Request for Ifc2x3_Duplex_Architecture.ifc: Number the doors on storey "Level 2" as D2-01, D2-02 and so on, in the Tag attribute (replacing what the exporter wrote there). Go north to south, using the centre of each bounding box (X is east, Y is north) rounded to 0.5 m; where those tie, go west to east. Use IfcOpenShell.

First a look at what the model holds.

```python
import ifcopenshell
import ifcopenshell.util.element
import ifcopenshell.util.placement

model = ifcopenshell.open("Ifc2x3_Duplex_Architecture.ifc")
print(model.schema)
storey = next(s for s in model.by_type("IfcBuildingStorey") if s.Name == "Level 2")
doors = [e for e in ifcopenshell.util.element.get_decomposition(storey) if e.is_a("IfcDoor")]
for e in sorted(doors, key=lambda e: e.id()):
    origin = ifcopenshell.util.placement.get_local_placement(e.ObjectPlacement)[:3, 3]
    print(e.id(), e.Tag, e.Name, origin.round(2) + 0.0, sep=" | ")
```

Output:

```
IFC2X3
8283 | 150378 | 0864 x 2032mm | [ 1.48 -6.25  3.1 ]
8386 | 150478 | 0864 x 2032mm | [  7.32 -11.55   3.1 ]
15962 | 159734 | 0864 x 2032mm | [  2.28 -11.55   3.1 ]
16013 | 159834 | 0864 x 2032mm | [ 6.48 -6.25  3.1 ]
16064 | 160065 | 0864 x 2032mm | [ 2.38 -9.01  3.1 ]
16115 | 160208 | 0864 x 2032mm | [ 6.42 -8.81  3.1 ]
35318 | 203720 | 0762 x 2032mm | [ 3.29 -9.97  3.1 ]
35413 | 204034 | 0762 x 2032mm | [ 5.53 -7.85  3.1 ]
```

```python
import ifcopenshell
import ifcopenshell.geom
import ifcopenshell.util.element
import ifcopenshell.util.shape

model = ifcopenshell.open("Ifc2x3_Duplex_Architecture.ifc")
settings = ifcopenshell.geom.settings()
settings.set("use-world-coords", True)


def centre(element):
    shape = ifcopenshell.geom.create_shape(settings, element)
    return ifcopenshell.util.shape.get_bbox_centroid(shape.geometry)


storey = next(s for s in model.by_type("IfcBuildingStorey") if s.Name == "Level 2")
doors = [e for e in ifcopenshell.util.element.get_decomposition(storey) if e.is_a("IfcDoor")]

# Insertion points can sit at a corner or the storey origin, so sort by the geometry (in metres).
centres = {e: centre(e) for e in doors}
doors.sort(key=lambda e: (-round(centres[e][1] / 0.5), centres[e][0]))

for i, e in enumerate(doors, start=1):
    number = f"D2-{i:02d}"
    e.Tag = number
    print(e.id(), number)

model.write("Ifc2x3_Duplex_Architecture-out.ifc")
```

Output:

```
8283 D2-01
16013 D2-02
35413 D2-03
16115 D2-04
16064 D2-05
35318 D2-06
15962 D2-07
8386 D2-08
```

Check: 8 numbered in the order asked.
